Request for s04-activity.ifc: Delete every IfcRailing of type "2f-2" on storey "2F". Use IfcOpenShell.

First a look at what the model holds.

```python
import ifcopenshell
import ifcopenshell.util.element

model = ifcopenshell.open("s04-activity.ifc")
print(model.schema)
storey = next(s for s in model.by_type("IfcBuildingStorey") if s.Name == "2F")
railings = [e for e in ifcopenshell.util.element.get_decomposition(storey) if e.is_a("IfcRailing")]
seen = {}
for e in railings:
    element_type = ifcopenshell.util.element.get_type(e)
    name = element_type.Name if element_type not in (None, e) else None
    seen[name] = seen.get(name, 0) + 1
for name, count in sorted(seen.items(), key=str):
    print(count, "x", name)
```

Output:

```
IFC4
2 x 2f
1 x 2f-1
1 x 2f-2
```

```python
import ifcopenshell
import ifcopenshell.api.root
import ifcopenshell.util.element

model = ifcopenshell.open("s04-activity.ifc")

storey = next(s for s in model.by_type("IfcBuildingStorey") if s.Name == "2F")
railings = [e for e in ifcopenshell.util.element.get_decomposition(storey) if e.is_a("IfcRailing")]
targets = [e for e in railings if (t := ifcopenshell.util.element.get_type(e)) not in (None, e) and t.Name == "2f-2"]

for e in targets:
    ifcopenshell.api.root.remove_product(model, product=e)
print(len(targets), "removed")

model.write("s04-activity-out.ifc")
```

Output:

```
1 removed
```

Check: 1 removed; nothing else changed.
